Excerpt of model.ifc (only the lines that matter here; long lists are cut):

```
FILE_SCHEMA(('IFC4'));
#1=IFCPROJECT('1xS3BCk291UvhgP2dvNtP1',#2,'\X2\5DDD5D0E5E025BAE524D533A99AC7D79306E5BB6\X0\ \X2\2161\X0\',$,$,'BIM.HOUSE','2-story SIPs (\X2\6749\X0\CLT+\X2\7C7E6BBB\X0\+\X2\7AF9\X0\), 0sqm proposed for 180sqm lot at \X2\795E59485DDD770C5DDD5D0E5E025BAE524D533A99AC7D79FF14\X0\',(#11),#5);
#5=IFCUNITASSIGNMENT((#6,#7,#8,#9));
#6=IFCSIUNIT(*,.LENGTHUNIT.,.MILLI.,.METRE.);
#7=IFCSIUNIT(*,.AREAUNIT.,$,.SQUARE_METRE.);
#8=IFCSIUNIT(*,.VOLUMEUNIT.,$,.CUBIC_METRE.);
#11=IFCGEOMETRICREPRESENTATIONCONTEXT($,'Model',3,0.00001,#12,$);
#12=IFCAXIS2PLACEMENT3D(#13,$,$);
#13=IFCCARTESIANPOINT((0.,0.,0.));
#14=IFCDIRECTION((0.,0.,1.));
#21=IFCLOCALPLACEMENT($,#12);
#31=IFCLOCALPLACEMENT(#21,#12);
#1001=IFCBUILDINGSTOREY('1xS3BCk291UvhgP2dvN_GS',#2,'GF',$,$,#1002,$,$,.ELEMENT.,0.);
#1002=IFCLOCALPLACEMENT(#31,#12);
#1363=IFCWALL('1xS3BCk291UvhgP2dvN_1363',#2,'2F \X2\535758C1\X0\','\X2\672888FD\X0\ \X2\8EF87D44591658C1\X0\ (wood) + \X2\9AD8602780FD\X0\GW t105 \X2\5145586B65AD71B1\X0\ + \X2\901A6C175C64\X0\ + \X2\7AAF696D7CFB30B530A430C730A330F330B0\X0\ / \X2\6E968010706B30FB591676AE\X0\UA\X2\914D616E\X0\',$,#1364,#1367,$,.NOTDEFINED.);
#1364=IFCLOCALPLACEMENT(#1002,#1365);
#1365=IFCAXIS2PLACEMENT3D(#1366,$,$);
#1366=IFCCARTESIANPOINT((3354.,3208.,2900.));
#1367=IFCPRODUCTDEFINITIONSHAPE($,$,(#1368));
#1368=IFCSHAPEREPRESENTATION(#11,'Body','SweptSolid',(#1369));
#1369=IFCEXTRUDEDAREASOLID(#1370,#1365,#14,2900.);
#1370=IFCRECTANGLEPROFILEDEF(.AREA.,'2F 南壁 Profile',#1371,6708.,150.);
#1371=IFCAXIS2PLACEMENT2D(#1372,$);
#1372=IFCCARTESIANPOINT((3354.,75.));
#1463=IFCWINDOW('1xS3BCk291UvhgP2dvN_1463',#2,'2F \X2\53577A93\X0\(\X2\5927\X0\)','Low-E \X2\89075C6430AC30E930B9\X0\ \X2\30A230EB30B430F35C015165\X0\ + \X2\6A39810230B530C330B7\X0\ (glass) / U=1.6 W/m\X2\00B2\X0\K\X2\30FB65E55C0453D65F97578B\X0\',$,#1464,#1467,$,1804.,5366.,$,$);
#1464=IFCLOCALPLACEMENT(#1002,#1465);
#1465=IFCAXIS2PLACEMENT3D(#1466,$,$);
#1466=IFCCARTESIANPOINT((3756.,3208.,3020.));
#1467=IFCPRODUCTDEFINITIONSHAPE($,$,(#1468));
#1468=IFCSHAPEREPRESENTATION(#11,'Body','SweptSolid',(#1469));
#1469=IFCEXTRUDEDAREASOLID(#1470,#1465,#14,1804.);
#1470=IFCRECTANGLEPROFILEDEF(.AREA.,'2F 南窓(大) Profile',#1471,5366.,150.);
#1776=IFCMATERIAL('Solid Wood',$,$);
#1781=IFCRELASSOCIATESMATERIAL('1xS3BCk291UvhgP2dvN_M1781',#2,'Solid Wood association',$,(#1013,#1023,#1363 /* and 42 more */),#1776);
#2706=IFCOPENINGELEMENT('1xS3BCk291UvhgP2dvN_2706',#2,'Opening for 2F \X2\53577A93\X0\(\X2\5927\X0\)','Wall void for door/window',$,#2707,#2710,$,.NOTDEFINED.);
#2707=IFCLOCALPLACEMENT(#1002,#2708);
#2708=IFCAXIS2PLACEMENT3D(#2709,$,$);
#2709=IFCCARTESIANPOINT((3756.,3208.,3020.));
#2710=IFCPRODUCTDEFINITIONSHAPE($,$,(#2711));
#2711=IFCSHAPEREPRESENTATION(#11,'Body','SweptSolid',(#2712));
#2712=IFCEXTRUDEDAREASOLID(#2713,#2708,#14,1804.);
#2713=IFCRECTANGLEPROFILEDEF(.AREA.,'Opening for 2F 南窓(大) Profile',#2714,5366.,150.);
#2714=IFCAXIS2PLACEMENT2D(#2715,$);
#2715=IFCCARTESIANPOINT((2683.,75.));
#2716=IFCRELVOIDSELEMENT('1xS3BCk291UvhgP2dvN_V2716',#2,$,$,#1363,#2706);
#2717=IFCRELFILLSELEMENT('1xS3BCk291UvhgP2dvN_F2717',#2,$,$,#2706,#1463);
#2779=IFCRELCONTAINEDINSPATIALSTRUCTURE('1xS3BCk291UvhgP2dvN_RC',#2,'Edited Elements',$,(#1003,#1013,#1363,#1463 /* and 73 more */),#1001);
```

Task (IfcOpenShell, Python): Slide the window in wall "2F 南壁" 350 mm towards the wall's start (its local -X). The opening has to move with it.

```python
import ifcopenshell
import ifcopenshell.api.geometry
import ifcopenshell.util.placement
import ifcopenshell.util.unit

model = ifcopenshell.open("model.ifc")
unit_scale = ifcopenshell.util.unit.calculate_unit_scale(model)

window = model.by_guid("1xS3BCk291UvhgP2dvN_1463")
opening = window.FillsVoids[0].RelatingOpeningElement
wall = opening.VoidsElements[0].RelatingBuildingElement

wall_matrix = ifcopenshell.util.placement.get_local_placement(wall.ObjectPlacement)
shift = wall_matrix[:3, 0] * -0.35 / unit_scale
before = ifcopenshell.util.placement.get_local_placement(window.ObjectPlacement)[:3, 3].copy()

# The window is not placed relative to its opening, so move both.
for product in (opening, window):
    matrix = ifcopenshell.util.placement.get_local_placement(product.ObjectPlacement)
    matrix[:3, 3] += shift
    ifcopenshell.api.geometry.edit_object_placement(model, product=product, matrix=matrix, is_si=False)

after = ifcopenshell.util.placement.get_local_placement(window.ObjectPlacement)[:3, 3]
print("window moved by", (after - before).round(3) + 0.0)

model.write("model_v2.ifc")
```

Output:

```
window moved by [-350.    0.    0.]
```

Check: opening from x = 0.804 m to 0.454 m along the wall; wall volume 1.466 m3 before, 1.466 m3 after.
